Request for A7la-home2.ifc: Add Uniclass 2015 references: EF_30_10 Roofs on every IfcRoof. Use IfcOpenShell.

First a look at what the model holds.

```python
import ifcopenshell

model = ifcopenshell.open("A7la-home2.ifc")
print(model.schema)
print("classifications:", [c.Name for c in model.by_type("IfcClassification")])
for ifc_class in ("IfcDoor", "IfcRoof", "IfcStair", "IfcWall", "IfcWindow"):
    print(ifc_class, len(model.by_type(ifc_class)))
```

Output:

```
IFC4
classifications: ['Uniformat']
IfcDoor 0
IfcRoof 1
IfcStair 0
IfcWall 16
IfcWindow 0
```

```python
import ifcopenshell
import ifcopenshell.api.classification

model = ifcopenshell.open("A7la-home2.ifc")

system = ifcopenshell.api.classification.add_classification(model, classification="Uniclass 2015")

codes = {
    "IfcRoof": ("EF_30_10", "Roofs"),
}
for ifc_class, (code, name) in codes.items():
    products = model.by_type(ifc_class)
    ifcopenshell.api.classification.add_reference(
        model, products=products, classification=system, identification=code, name=name
    )
    print(code, len(products))

model.write("A7la-home2_rev.ifc")
```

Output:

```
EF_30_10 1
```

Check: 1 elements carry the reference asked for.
